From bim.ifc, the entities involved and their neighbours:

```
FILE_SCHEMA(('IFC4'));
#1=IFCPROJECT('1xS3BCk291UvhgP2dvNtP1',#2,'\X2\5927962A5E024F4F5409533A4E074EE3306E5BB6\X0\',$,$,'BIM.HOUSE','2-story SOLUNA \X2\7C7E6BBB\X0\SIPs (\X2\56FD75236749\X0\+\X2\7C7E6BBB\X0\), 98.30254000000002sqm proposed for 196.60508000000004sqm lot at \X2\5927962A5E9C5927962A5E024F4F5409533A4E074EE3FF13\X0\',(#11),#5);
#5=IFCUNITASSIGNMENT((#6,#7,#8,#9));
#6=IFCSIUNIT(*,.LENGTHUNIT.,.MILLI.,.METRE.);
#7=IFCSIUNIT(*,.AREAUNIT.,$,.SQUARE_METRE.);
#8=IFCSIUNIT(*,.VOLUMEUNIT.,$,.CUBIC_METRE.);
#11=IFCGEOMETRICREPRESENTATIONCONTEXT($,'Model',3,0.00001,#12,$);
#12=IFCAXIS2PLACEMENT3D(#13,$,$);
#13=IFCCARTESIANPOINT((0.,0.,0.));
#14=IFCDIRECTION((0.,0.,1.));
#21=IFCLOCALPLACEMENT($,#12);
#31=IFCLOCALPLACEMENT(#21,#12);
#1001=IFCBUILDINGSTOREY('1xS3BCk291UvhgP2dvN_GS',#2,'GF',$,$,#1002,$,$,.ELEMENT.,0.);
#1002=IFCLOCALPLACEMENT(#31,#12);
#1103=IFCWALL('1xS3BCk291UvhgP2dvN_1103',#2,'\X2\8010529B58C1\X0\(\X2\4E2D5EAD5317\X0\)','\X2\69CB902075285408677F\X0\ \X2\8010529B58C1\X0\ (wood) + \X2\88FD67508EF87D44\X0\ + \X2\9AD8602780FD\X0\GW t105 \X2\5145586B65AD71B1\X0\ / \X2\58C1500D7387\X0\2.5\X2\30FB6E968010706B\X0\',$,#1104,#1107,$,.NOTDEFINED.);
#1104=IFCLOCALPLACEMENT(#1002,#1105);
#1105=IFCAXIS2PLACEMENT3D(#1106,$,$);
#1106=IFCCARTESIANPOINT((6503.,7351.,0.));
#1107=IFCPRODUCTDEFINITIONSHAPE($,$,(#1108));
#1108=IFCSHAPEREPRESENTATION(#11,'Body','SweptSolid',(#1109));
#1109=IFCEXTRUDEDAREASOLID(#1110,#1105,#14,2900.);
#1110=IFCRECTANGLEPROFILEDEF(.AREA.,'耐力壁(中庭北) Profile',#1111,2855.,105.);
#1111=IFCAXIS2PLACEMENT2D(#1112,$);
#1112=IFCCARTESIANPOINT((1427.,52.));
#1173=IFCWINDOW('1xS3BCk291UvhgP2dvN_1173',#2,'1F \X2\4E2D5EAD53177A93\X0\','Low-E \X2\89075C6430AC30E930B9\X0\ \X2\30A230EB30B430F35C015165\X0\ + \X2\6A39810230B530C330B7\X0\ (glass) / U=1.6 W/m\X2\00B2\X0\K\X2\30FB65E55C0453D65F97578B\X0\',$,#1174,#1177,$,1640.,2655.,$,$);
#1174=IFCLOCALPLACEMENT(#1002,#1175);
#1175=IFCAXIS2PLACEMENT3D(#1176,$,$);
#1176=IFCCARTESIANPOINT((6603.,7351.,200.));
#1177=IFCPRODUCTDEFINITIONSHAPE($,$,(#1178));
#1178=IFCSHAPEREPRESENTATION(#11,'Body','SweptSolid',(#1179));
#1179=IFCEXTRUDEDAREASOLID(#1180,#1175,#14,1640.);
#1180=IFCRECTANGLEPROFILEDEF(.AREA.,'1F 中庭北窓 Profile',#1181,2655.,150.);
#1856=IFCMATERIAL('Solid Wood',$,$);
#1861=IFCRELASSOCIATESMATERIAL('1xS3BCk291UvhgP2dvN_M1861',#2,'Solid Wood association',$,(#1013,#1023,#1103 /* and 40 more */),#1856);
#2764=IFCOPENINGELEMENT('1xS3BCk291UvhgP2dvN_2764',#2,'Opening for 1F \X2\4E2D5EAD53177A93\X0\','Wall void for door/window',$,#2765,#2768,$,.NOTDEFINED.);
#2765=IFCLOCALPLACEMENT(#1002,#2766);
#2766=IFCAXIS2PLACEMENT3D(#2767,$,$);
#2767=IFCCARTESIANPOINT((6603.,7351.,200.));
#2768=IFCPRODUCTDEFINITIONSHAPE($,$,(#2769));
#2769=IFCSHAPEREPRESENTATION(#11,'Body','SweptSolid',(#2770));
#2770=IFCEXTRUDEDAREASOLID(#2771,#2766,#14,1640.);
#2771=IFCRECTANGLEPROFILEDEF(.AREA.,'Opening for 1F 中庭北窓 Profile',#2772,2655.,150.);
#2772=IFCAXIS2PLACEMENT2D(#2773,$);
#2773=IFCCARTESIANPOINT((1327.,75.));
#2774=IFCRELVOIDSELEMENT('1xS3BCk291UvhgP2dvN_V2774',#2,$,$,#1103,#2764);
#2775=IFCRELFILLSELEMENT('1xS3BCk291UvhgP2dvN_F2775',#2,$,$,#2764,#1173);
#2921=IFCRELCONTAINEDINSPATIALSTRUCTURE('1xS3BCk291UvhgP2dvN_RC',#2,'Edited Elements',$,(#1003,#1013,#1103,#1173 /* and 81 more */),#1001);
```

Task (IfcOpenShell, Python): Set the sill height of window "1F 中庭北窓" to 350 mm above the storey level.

```python
import numpy as np
import ifcopenshell
import ifcopenshell.api.geometry
import ifcopenshell.geom
import ifcopenshell.util.element
import ifcopenshell.util.placement
import ifcopenshell.util.shape
import ifcopenshell.util.unit

model = ifcopenshell.open("bim.ifc")
unit_scale = ifcopenshell.util.unit.calculate_unit_scale(model)

window = model.by_id(1173)
opening = window.FillsVoids[0].RelatingOpeningElement
storey = ifcopenshell.util.element.get_container(window, ifc_class="IfcBuildingStorey")
level = ifcopenshell.util.placement.get_local_placement(storey.ObjectPlacement)[2, 3]

# The opening's origin need not be at the sill, so measure its lowest point.
shape = ifcopenshell.geom.create_shape(ifcopenshell.geom.settings(), opening)
bottom = ifcopenshell.util.shape.get_shape_bottom_elevation(shape, shape.geometry) / unit_scale
dz = level + 0.35 / unit_scale - bottom

shift = np.array([0.0, 0.0, dz])
# The window is not placed relative to its opening, so move both.
for product in (opening, window):
    matrix = ifcopenshell.util.placement.get_local_placement(product.ObjectPlacement)
    matrix[:3, 3] += shift
    ifcopenshell.api.geometry.edit_object_placement(model, product=product, matrix=matrix, is_si=False)

print(f"moved by {dz * unit_scale:+.3f} m")

model.write("bim_updated.ifc")
```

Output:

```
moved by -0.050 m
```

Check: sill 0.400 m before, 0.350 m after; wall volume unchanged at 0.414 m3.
